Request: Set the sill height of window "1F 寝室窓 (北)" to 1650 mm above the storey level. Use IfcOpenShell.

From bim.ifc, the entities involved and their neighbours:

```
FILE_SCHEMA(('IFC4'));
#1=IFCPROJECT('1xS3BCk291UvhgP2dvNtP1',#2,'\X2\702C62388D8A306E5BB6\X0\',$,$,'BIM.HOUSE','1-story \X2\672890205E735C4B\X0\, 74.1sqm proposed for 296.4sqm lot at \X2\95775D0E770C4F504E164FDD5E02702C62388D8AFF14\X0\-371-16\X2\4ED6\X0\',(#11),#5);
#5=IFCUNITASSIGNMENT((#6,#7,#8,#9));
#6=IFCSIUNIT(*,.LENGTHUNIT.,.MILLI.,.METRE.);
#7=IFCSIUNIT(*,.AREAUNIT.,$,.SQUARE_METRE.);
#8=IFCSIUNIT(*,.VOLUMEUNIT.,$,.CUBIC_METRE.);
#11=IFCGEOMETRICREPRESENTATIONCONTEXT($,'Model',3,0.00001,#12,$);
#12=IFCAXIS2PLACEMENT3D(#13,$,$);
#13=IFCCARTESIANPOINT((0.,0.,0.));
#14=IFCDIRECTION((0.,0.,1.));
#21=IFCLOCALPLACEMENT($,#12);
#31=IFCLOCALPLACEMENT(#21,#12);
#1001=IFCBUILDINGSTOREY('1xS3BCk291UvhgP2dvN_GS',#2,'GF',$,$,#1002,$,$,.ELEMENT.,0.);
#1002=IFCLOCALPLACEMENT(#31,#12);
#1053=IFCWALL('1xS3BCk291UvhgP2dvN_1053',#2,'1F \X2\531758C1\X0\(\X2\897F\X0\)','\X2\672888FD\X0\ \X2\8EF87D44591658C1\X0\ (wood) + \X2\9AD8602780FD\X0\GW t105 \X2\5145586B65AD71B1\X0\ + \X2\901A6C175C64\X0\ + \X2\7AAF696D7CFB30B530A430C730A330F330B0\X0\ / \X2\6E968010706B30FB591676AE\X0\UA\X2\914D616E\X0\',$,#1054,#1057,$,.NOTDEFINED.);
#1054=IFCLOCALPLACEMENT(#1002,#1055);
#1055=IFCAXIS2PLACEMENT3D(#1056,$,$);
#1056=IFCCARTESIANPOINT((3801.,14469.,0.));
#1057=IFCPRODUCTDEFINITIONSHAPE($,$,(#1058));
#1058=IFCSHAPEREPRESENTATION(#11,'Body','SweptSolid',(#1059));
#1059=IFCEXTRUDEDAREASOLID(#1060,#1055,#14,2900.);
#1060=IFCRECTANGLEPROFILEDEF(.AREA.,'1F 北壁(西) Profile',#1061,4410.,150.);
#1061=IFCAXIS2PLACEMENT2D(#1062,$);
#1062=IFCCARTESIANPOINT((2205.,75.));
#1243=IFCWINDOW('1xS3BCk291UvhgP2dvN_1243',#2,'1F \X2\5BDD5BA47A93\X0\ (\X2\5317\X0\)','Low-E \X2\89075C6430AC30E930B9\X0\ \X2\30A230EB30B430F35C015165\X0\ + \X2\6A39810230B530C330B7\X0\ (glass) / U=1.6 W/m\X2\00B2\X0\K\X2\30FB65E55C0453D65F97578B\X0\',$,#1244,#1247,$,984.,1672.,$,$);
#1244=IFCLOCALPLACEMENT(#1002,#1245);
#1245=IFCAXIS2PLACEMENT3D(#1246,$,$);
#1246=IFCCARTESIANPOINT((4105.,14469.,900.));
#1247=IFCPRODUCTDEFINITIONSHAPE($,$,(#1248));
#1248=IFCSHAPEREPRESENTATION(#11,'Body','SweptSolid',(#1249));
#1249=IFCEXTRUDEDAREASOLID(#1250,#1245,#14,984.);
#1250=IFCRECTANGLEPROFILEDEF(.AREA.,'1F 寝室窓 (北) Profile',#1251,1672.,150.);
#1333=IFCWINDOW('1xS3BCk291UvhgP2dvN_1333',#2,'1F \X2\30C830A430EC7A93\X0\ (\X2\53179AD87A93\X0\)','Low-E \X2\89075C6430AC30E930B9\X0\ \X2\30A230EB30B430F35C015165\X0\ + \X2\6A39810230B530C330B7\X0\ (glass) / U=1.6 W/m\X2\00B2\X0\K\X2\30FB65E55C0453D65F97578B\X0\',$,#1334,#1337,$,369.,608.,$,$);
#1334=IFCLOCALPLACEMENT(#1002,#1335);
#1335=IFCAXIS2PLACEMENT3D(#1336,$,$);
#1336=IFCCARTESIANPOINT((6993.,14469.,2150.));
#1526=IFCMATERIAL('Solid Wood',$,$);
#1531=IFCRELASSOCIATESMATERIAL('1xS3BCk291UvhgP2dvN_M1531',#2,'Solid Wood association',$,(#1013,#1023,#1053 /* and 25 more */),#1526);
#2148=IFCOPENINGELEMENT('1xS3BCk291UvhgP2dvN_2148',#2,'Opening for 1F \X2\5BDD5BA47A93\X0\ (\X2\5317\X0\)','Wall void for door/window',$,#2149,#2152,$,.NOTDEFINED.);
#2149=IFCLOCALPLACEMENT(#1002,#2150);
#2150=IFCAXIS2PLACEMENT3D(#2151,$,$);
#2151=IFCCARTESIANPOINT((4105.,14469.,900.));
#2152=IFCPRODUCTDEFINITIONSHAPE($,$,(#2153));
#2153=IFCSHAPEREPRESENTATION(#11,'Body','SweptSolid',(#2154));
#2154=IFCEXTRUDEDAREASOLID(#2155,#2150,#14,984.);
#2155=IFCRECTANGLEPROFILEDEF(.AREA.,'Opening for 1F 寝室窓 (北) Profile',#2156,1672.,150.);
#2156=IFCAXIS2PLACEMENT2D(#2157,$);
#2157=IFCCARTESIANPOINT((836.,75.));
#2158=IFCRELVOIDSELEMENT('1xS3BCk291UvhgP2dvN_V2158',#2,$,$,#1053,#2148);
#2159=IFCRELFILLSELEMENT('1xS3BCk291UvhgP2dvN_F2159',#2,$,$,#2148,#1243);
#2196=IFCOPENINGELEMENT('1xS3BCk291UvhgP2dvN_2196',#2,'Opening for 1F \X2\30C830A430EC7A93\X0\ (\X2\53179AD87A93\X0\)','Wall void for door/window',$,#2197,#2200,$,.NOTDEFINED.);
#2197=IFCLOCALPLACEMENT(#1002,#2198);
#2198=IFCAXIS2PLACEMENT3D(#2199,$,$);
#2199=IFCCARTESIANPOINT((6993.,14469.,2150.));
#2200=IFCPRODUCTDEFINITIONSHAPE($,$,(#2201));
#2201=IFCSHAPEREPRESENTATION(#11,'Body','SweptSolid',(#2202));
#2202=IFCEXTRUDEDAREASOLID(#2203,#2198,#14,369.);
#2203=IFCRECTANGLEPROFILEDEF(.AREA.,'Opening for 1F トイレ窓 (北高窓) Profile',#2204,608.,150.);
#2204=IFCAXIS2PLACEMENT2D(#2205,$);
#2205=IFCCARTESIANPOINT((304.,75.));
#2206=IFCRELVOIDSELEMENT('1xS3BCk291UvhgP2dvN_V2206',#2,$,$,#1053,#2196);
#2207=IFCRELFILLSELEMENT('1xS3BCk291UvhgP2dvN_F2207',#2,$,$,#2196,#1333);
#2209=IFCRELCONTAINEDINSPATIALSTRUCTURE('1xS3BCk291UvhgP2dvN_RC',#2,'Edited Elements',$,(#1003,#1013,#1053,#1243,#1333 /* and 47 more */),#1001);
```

```python
import numpy as np
import ifcopenshell
import ifcopenshell.api.geometry
import ifcopenshell.geom
import ifcopenshell.util.element
import ifcopenshell.util.placement
import ifcopenshell.util.shape
import ifcopenshell.util.unit

model = ifcopenshell.open("bim.ifc")
unit_scale = ifcopenshell.util.unit.calculate_unit_scale(model)

window = model.by_id(1243)
opening = window.FillsVoids[0].RelatingOpeningElement
storey = ifcopenshell.util.element.get_container(window, ifc_class="IfcBuildingStorey")
level = ifcopenshell.util.placement.get_local_placement(storey.ObjectPlacement)[2, 3]

# The opening's origin need not be at the sill, so measure its lowest point.
shape = ifcopenshell.geom.create_shape(ifcopenshell.geom.settings(), opening)
bottom = ifcopenshell.util.shape.get_shape_bottom_elevation(shape, shape.geometry) / unit_scale
dz = level + 1650.0 - bottom

shift = np.array([0.0, 0.0, dz])
# The window is not placed relative to its opening, so move both.
for product in (opening, window):
    matrix = ifcopenshell.util.placement.get_local_placement(product.ObjectPlacement)
    matrix[:3, 3] += shift
    ifcopenshell.api.geometry.edit_object_placement(model, product=product, matrix=matrix, is_si=False)

print(f"moved by {dz * unit_scale:+.3f} m")

model.write("bim_v2.ifc")
```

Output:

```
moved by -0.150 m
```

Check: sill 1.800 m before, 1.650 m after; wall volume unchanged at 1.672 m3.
